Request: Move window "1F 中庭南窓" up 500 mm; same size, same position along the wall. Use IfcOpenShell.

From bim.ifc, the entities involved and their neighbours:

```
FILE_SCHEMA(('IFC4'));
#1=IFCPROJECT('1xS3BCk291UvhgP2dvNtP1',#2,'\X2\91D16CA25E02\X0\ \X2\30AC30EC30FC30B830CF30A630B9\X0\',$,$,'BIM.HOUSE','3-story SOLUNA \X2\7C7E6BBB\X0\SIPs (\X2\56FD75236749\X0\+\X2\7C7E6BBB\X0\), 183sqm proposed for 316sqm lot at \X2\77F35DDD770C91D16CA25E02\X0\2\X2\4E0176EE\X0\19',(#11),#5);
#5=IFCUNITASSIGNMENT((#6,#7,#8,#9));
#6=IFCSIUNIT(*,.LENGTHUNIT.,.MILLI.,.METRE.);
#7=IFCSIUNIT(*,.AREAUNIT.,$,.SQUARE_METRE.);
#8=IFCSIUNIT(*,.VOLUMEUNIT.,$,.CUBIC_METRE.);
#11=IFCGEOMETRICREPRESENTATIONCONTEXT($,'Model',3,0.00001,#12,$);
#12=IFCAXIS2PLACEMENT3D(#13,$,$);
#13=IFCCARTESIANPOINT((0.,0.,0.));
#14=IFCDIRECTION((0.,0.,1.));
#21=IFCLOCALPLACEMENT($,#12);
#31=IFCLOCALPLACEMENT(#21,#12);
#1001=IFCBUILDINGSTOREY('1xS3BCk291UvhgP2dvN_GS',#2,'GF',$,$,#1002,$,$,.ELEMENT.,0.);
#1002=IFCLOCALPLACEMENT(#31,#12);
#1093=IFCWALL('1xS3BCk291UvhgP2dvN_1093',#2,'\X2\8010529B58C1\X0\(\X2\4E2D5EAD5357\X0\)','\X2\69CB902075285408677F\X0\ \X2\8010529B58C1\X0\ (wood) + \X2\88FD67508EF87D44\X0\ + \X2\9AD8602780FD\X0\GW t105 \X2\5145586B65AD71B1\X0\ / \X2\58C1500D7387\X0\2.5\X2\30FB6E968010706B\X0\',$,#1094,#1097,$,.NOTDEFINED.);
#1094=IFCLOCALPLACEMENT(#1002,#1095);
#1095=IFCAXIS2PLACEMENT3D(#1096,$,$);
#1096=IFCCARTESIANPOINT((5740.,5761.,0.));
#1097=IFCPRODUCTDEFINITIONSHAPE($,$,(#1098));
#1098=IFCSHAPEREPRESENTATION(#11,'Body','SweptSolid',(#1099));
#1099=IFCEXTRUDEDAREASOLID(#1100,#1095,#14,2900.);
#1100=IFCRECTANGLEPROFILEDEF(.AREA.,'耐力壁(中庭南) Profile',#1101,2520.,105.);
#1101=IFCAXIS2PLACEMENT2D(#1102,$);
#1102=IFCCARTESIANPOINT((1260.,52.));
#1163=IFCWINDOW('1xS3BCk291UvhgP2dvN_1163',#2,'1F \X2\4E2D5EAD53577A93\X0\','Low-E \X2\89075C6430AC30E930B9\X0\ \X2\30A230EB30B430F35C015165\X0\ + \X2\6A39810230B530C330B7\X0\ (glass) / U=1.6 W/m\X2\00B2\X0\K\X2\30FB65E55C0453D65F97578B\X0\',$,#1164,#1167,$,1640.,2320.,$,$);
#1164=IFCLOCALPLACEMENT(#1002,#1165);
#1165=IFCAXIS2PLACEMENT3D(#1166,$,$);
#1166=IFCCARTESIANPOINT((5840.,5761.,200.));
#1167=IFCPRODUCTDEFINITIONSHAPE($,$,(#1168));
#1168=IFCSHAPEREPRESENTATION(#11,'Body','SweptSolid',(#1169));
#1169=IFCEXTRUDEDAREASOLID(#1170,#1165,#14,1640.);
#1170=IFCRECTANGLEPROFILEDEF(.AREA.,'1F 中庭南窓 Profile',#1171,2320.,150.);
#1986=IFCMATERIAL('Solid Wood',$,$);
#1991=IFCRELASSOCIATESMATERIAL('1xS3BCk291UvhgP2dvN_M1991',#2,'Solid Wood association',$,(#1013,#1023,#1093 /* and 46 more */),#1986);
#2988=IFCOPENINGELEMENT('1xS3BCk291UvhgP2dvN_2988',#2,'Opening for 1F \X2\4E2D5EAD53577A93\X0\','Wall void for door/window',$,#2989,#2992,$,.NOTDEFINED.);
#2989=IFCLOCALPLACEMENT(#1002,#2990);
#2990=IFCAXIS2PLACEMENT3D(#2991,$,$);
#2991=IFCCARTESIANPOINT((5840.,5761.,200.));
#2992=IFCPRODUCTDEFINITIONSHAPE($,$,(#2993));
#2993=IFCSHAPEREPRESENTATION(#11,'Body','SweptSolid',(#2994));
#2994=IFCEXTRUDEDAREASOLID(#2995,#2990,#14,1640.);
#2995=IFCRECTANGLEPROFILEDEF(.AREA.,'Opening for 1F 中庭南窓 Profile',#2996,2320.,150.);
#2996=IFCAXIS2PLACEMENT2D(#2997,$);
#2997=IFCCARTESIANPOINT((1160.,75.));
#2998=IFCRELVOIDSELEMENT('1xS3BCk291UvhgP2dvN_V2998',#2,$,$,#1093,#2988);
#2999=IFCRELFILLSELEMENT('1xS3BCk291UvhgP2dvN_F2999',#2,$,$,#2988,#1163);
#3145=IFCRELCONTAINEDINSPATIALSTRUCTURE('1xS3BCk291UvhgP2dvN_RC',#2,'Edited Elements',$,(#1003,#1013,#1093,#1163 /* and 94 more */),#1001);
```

```python
import numpy as np
import ifcopenshell
import ifcopenshell.api.geometry
import ifcopenshell.util.placement
import ifcopenshell.util.unit

model = ifcopenshell.open("bim.ifc")
unit_scale = ifcopenshell.util.unit.calculate_unit_scale(model)

window = model.by_id(1163)
opening = window.FillsVoids[0].RelatingOpeningElement
dz = 0.5 / unit_scale

shift = np.array([0.0, 0.0, dz])
# The window is not placed relative to its opening, so move both.
for product in (opening, window):
    matrix = ifcopenshell.util.placement.get_local_placement(product.ObjectPlacement)
    matrix[:3, 3] += shift
    ifcopenshell.api.geometry.edit_object_placement(model, product=product, matrix=matrix, is_si=False)

print(f"moved by {dz * unit_scale:+.3f} m")

model.write("bim-out.ifc")
```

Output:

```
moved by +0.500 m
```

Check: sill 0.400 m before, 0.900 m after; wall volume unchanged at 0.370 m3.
